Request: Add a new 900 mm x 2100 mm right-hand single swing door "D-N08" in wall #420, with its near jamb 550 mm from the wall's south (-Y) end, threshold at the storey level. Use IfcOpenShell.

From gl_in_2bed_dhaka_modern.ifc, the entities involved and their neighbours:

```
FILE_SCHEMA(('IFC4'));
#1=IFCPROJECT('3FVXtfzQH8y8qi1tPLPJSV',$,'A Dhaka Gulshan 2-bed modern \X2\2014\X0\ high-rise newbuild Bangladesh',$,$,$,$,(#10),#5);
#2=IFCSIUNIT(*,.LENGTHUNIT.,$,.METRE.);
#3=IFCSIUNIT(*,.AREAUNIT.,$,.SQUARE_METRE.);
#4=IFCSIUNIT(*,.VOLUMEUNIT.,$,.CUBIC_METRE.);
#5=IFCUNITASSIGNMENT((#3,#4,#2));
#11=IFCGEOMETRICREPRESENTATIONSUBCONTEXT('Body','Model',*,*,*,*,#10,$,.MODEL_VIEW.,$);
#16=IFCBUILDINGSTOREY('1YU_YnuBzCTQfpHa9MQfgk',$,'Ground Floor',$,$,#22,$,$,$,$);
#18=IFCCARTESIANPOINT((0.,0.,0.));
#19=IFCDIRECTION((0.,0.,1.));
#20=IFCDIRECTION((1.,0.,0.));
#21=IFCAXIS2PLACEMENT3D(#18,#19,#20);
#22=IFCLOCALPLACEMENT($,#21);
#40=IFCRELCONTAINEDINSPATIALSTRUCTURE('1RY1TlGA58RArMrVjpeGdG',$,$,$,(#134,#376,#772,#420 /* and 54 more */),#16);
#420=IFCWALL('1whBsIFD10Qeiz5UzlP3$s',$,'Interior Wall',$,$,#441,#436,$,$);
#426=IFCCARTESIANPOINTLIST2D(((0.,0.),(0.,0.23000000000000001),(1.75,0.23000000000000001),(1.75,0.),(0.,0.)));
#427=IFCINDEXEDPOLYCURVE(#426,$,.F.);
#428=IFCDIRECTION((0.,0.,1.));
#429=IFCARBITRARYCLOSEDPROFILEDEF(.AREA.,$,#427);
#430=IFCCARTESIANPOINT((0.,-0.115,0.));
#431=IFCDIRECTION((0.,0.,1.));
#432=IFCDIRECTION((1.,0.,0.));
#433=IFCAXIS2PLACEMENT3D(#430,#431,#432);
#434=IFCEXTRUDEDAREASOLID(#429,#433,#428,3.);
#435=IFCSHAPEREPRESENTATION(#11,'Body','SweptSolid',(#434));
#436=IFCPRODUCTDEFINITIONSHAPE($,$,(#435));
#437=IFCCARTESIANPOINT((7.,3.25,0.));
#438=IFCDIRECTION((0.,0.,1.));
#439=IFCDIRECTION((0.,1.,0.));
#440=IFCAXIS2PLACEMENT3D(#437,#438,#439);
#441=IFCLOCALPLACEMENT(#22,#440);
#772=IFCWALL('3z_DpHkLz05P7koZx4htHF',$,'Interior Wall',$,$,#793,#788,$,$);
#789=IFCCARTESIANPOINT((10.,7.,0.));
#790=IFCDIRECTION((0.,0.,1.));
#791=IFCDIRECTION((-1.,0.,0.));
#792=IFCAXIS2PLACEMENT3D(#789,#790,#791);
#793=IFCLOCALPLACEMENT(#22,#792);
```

```python
import numpy as np
import ifcopenshell
import ifcopenshell.api.feature
import ifcopenshell.api.geometry
import ifcopenshell.api.root
import ifcopenshell.api.spatial
import ifcopenshell.geom
import ifcopenshell.util.element
import ifcopenshell.util.placement
import ifcopenshell.util.representation
import ifcopenshell.util.shape
import ifcopenshell.util.unit

model = ifcopenshell.open("gl_in_2bed_dhaka_modern.ifc")
unit_scale = ifcopenshell.util.unit.calculate_unit_scale(model)
settings = ifcopenshell.geom.settings()


def volume(element):
    """Net volume in cubic metres, openings subtracted."""
    shape = ifcopenshell.geom.create_shape(settings, element)
    return ifcopenshell.util.shape.get_volume(shape.geometry)


wall = model.by_guid("1whBsIFD10Qeiz5UzlP3$s")
storey = ifcopenshell.util.element.get_container(wall, ifc_class="IfcBuildingStorey")
context = ifcopenshell.util.representation.get_context(model, "Model", "Body", "MODEL_VIEW")
before = volume(wall)

width, height, from_end, sill = 0.9, 2.1, 0.55, 0.0  # metres

# The wall runs along its own X axis, and the end named is its -X end.
wall_shape = ifcopenshell.geom.create_shape(settings, wall)
x, y, z = ifcopenshell.util.shape.get_vertices(wall_shape.geometry).T
start = x.min() + from_end
face, thickness = float(y.min()), float(y.max() - y.min())
wall_matrix = ifcopenshell.util.placement.get_local_placement(wall.ObjectPlacement)
level = ifcopenshell.util.placement.get_local_placement(storey.ObjectPlacement)[2, 3]


def in_wall(x, y):
    """Placement at x, y metres in the wall's axes, at sill height."""
    matrix = wall_matrix.copy()
    matrix[:, 3] = wall_matrix @ np.array([x / unit_scale, y / unit_scale, 0.0, 1.0])
    matrix[2, 3] = level + sill / unit_scale
    return matrix


# Opening: a box that overshoots both wall faces by 50 mm.
opening = ifcopenshell.api.root.create_entity(model, ifc_class="IfcOpeningElement", predefined_type="OPENING")
box = ifcopenshell.api.geometry.add_wall_representation(
    model, context=context, length=width, height=height, thickness=thickness + 0.1
)
ifcopenshell.api.geometry.assign_representation(model, product=opening, representation=box)
ifcopenshell.api.geometry.edit_object_placement(model, product=opening, matrix=in_wall(start, face - 0.05), is_si=False)
ifcopenshell.api.feature.add_feature(model, feature=opening, element=wall)

door = ifcopenshell.api.root.create_entity(model, ifc_class="IfcDoor", name="D-N08", predefined_type="DOOR")
door.OverallWidth, door.OverallHeight = width / unit_scale, height / unit_scale
door.OperationType = "SINGLE_SWING_RIGHT"
body = ifcopenshell.api.geometry.add_door_representation(
    model,
    context=context,
    overall_width=door.OverallWidth,
    overall_height=door.OverallHeight,
    operation_type="SINGLE_SWING_RIGHT",
    lining_properties={"LiningDepth": thickness / unit_scale, "ThresholdDepth": thickness / unit_scale},
)
ifcopenshell.api.geometry.assign_representation(model, product=door, representation=body)
ifcopenshell.api.spatial.assign_container(model, products=[door], relating_structure=storey)
ifcopenshell.api.feature.add_filling(model, opening=opening, element=door)

# The lining spans the wall, so the door starts at the wall face.
ifcopenshell.api.geometry.edit_object_placement(model, product=door, matrix=in_wall(start, face), is_si=False)

after = volume(wall)

print(f"wall volume {before:.3f} -> {after:.3f} m3")

model.write("gl_in_2bed_dhaka_modern_edited.ifc")
```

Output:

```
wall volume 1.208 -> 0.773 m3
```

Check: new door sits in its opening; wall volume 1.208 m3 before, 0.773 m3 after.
